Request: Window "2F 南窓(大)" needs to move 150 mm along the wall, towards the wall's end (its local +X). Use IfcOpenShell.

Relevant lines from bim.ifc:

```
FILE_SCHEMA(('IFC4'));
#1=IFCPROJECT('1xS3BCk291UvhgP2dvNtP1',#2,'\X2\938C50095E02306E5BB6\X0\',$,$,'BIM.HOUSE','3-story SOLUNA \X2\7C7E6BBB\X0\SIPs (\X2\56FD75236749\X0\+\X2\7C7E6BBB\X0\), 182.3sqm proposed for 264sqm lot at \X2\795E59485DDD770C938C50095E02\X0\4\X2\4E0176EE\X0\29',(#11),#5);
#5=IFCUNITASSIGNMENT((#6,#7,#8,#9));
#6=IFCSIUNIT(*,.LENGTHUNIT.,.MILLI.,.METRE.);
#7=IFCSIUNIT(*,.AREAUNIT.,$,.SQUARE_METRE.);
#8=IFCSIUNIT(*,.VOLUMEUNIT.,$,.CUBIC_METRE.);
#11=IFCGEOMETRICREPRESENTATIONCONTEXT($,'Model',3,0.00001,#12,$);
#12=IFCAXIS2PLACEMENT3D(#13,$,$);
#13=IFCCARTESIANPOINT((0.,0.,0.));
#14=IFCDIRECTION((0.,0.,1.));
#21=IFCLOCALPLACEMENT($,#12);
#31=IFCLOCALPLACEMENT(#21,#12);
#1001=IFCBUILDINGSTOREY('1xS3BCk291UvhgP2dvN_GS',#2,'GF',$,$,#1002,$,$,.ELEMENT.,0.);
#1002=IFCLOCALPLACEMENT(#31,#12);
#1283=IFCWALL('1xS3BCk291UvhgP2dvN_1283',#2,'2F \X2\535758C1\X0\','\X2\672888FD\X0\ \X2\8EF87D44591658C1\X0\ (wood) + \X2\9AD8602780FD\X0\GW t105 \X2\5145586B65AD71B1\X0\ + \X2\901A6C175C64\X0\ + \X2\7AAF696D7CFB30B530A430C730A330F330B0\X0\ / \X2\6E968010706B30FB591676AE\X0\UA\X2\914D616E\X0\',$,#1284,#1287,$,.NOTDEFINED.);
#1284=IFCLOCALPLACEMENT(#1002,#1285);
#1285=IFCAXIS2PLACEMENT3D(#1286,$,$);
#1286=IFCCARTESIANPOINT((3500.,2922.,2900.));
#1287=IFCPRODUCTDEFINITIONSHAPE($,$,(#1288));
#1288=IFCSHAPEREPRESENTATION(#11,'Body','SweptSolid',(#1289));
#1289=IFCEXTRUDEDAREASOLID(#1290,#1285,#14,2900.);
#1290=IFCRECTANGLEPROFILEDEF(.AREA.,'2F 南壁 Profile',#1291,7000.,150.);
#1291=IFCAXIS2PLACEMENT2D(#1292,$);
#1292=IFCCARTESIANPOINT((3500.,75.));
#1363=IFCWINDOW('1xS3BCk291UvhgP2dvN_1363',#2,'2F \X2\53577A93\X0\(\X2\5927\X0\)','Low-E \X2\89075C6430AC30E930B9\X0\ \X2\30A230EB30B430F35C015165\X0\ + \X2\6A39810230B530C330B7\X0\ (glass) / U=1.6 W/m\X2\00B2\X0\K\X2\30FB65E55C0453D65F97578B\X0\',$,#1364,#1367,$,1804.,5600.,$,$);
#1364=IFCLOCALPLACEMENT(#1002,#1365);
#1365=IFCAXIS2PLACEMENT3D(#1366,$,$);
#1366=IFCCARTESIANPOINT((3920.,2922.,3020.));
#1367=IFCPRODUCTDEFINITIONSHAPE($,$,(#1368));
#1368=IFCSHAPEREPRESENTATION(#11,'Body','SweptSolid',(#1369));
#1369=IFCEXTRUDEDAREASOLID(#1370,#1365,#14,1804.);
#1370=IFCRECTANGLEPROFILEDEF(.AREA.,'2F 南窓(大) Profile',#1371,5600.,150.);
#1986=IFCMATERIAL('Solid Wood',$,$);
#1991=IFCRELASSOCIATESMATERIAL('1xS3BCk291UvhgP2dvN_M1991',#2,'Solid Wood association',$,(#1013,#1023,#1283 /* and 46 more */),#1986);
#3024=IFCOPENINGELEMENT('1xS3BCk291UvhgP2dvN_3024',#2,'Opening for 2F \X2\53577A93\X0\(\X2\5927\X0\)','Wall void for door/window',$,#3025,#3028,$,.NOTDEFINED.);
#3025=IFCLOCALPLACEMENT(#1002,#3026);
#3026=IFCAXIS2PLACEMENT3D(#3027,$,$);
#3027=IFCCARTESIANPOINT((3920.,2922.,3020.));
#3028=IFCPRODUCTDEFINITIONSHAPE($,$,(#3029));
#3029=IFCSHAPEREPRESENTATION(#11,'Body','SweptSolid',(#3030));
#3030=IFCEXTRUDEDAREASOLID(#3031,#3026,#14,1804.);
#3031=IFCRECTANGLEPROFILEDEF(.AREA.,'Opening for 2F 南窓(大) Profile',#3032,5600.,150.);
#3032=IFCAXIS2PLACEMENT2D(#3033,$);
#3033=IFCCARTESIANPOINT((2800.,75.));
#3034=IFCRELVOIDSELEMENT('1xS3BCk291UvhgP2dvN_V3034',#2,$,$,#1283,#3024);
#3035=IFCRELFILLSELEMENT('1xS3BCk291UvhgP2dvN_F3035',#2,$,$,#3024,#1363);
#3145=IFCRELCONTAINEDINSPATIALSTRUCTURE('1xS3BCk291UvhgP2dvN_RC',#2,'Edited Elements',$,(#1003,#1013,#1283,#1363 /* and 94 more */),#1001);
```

```python
import ifcopenshell
import ifcopenshell.api.geometry
import ifcopenshell.util.placement
import ifcopenshell.util.unit

model = ifcopenshell.open("bim.ifc")
unit_scale = ifcopenshell.util.unit.calculate_unit_scale(model)

window = model.by_id(1363)
opening = window.FillsVoids[0].RelatingOpeningElement
wall = opening.VoidsElements[0].RelatingBuildingElement

wall_matrix = ifcopenshell.util.placement.get_local_placement(wall.ObjectPlacement)
shift = wall_matrix[:3, 0] * 0.15 / unit_scale
before = ifcopenshell.util.placement.get_local_placement(window.ObjectPlacement)[:3, 3].copy()

# The window is not placed relative to its opening, so move both.
for product in (opening, window):
    matrix = ifcopenshell.util.placement.get_local_placement(product.ObjectPlacement)
    matrix[:3, 3] += shift
    ifcopenshell.api.geometry.edit_object_placement(model, product=product, matrix=matrix, is_si=False)

after = ifcopenshell.util.placement.get_local_placement(window.ObjectPlacement)[:3, 3]
print("window moved by", (after - before).round(3) + 0.0)

model.write("bim-out.ifc")
```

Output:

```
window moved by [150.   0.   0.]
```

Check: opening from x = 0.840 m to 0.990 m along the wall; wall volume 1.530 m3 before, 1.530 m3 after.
